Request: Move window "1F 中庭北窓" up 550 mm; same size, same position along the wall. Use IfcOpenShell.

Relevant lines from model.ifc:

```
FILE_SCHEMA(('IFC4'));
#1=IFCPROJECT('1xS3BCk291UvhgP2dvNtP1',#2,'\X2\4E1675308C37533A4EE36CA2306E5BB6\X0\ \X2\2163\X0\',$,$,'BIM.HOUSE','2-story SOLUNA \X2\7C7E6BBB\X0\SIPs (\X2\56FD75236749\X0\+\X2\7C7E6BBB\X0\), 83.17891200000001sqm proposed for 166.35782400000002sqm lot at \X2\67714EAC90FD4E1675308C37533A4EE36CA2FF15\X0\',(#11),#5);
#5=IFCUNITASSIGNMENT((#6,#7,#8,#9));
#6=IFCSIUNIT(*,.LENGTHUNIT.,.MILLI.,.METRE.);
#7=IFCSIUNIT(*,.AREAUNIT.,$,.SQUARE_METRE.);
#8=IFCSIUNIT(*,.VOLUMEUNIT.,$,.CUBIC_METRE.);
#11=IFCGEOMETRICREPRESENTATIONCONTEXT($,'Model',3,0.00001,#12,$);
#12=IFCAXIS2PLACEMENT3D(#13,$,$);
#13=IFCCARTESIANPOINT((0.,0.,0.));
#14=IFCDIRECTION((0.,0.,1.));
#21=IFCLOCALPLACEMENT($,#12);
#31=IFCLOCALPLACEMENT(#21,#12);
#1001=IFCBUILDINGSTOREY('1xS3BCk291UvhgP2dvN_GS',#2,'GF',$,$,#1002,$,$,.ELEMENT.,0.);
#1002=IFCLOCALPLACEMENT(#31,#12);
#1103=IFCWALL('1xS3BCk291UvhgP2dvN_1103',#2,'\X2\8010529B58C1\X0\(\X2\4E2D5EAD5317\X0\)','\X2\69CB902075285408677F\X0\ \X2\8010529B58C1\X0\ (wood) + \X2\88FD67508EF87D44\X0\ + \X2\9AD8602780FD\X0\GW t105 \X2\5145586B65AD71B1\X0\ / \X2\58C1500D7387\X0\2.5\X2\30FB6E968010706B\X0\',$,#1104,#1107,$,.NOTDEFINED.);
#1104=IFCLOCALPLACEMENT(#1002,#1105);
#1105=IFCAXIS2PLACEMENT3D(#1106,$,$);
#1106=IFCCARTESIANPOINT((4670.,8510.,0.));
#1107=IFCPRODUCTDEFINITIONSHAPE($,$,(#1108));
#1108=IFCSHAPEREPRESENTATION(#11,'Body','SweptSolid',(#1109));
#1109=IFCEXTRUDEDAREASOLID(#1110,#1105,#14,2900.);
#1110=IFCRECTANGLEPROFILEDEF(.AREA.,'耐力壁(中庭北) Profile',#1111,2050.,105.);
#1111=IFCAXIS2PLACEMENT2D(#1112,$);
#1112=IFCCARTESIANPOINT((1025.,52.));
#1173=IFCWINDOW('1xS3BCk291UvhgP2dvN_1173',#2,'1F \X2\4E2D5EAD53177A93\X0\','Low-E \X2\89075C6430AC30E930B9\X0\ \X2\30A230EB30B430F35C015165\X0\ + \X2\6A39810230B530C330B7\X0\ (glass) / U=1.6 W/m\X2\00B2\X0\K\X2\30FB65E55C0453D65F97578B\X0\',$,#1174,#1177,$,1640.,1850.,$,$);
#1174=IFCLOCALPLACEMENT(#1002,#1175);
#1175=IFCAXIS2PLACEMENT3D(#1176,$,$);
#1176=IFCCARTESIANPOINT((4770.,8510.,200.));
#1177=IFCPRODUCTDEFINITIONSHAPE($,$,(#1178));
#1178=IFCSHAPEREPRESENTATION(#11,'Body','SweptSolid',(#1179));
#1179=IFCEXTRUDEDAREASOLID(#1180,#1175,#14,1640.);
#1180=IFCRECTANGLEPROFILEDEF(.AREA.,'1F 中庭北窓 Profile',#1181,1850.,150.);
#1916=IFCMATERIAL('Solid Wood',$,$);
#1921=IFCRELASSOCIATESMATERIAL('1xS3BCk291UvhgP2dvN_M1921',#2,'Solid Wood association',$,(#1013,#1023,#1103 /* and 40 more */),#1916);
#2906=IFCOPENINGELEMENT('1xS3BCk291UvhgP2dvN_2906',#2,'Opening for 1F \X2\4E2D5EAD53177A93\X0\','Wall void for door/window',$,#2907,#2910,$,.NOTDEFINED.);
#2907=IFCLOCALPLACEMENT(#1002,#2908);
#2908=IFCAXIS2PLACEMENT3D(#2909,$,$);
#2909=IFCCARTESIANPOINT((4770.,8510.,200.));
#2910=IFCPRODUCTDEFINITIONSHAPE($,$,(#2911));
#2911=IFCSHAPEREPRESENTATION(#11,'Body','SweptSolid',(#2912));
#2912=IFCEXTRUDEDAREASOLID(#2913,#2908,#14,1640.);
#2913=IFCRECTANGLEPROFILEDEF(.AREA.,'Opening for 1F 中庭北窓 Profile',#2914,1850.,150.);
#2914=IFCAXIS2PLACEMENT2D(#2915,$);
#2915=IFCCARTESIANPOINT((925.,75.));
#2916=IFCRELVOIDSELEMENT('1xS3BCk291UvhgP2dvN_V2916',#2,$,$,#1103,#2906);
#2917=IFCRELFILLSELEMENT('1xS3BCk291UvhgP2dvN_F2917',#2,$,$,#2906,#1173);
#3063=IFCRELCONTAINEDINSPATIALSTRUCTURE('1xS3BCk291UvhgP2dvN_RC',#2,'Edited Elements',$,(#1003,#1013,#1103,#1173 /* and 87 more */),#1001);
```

```python
import numpy as np
import ifcopenshell
import ifcopenshell.api.geometry
import ifcopenshell.util.placement
import ifcopenshell.util.unit

model = ifcopenshell.open("model.ifc")
unit_scale = ifcopenshell.util.unit.calculate_unit_scale(model)

window = model.by_id(1173)
opening = window.FillsVoids[0].RelatingOpeningElement
dz = 0.55 / unit_scale

shift = np.array([0.0, 0.0, dz])
# The window is not placed relative to its opening, so move both.
for product in (opening, window):
    matrix = ifcopenshell.util.placement.get_local_placement(product.ObjectPlacement)
    matrix[:3, 3] += shift
    ifcopenshell.api.geometry.edit_object_placement(model, product=product, matrix=matrix, is_si=False)

print(f"moved by {dz * unit_scale:+.3f} m")

model.write("model-out.ifc")
```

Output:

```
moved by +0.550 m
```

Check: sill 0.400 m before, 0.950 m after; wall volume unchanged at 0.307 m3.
